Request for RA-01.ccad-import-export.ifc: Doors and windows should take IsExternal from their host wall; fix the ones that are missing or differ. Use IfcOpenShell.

First a look at what the model holds.

```python
import ifcopenshell
import ifcopenshell.util.element

model = ifcopenshell.open("RA-01.ccad-import-export.ifc")
print(model.schema)
seen = {}
for e in model.by_type("IfcDoor") + model.by_type("IfcWindow"):
    if not e.FillsVoids:
        continue
    host = e.FillsVoids[0].RelatingOpeningElement.VoidsElements[0].RelatingBuildingElement
    own = ifcopenshell.util.element.get_pset(e, f"Pset_{e.is_a()[3:].removesuffix('StandardCase')}Common", "IsExternal")
    wall = ifcopenshell.util.element.get_pset(host, "Pset_WallCommon", "IsExternal")
    seen[e.is_a(), own, wall] = seen.get((e.is_a(), own, wall), 0) + 1
for (cls, own, wall), count in sorted(seen.items(), key=str):
    print(count, cls, "IsExternal:", own, "| host wall:", wall)
```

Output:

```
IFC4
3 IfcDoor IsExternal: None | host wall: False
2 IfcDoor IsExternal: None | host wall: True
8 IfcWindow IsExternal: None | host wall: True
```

```python
import ifcopenshell
import ifcopenshell.api.pset
import ifcopenshell.util.element

model = ifcopenshell.open("RA-01.ccad-import-export.ifc")

count = 0
for ifc_class, pset_name in (("IfcDoor", "Pset_DoorCommon"), ("IfcWindow", "Pset_WindowCommon")):
    for e in model.by_type(ifc_class):
        if not e.FillsVoids:
            continue
        host = e.FillsVoids[0].RelatingOpeningElement.VoidsElements[0].RelatingBuildingElement
        external = ifcopenshell.util.element.get_pset(host, "Pset_WallCommon", "IsExternal")
        if external is None or ifcopenshell.util.element.get_pset(e, pset_name, "IsExternal") == external:
            continue
        found = ifcopenshell.util.element.get_pset(e, pset_name, should_inherit=False)
        if found:
            pset = model.by_id(found["id"])
            if len(ifcopenshell.util.element.get_elements_by_pset(pset)) > 1:
                pset = ifcopenshell.api.pset.unshare_pset(model, products=[e], pset=pset)[0]
        else:
            pset = ifcopenshell.api.pset.add_pset(model, product=e, name=pset_name)
        ifcopenshell.api.pset.edit_pset(model, pset=pset, properties={"IsExternal": external})
        count += 1

print(count, "updated")

model.write("RA-01.ccad-import-export_edited.ifc")
```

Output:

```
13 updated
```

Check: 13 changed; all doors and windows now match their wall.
